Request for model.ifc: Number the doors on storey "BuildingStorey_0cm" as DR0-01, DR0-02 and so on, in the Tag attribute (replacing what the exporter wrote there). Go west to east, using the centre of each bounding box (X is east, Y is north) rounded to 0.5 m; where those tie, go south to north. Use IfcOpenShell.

First a look at what the model holds.

```python
import ifcopenshell
import ifcopenshell.util.element
import ifcopenshell.util.placement

model = ifcopenshell.open("model.ifc")
print(model.schema)
storey = next(s for s in model.by_type("IfcBuildingStorey") if s.Name == "BuildingStorey_0cm")
doors = [e for e in ifcopenshell.util.element.get_decomposition(storey) if e.is_a("IfcDoor")]
for e in sorted(doors, key=lambda e: e.id()):
    origin = ifcopenshell.util.placement.get_local_placement(e.ObjectPlacement)[:3, 3]
    print(e.id(), e.Tag, e.Name, origin.round(2) + 0.0, sep=" | ")
```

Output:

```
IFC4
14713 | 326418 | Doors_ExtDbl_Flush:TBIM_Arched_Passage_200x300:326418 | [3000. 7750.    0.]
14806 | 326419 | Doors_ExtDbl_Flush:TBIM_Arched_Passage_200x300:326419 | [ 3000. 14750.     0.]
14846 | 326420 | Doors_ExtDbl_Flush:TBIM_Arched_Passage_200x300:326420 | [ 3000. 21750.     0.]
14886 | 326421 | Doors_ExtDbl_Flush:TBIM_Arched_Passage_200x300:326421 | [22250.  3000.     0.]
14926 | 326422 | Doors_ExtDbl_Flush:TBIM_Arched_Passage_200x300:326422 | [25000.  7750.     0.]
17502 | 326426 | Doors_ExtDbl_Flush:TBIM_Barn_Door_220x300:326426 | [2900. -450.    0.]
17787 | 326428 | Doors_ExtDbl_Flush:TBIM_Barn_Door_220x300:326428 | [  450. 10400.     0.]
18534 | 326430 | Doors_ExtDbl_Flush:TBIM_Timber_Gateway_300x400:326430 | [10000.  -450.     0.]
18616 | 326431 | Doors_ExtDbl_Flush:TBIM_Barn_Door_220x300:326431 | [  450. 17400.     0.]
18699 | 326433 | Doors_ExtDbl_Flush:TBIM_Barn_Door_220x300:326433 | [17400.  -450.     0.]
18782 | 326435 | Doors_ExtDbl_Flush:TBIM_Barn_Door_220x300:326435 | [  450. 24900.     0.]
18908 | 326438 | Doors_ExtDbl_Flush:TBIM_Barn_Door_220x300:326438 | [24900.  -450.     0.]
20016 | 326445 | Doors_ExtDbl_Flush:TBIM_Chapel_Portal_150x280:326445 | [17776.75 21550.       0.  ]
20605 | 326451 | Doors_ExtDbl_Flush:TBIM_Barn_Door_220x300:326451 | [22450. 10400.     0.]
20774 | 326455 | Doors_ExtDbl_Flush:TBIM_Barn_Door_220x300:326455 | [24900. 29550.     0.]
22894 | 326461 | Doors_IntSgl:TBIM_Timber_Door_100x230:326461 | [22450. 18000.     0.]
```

```python
import ifcopenshell
import ifcopenshell.geom
import ifcopenshell.util.element
import ifcopenshell.util.shape

model = ifcopenshell.open("model.ifc")
settings = ifcopenshell.geom.settings()
settings.set("use-world-coords", True)


def centre(element):
    shape = ifcopenshell.geom.create_shape(settings, element)
    return ifcopenshell.util.shape.get_bbox_centroid(shape.geometry)


storey = next(s for s in model.by_type("IfcBuildingStorey") if s.Name == "BuildingStorey_0cm")
doors = [e for e in ifcopenshell.util.element.get_decomposition(storey) if e.is_a("IfcDoor")]

# Insertion points can sit at a corner or the storey origin, so sort by the geometry (in metres).
centres = {e: centre(e) for e in doors}
doors.sort(key=lambda e: (round(centres[e][0] / 0.5), centres[e][1]))

for i, e in enumerate(doors, start=1):
    number = f"DR0-{i:02d}"
    e.Tag = number
    print(e.id(), number)

model.write("model_updated.ifc")
```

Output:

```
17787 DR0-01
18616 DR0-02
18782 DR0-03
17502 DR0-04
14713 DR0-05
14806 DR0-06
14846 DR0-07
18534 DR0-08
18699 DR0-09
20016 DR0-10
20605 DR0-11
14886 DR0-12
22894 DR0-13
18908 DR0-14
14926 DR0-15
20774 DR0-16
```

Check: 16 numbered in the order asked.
